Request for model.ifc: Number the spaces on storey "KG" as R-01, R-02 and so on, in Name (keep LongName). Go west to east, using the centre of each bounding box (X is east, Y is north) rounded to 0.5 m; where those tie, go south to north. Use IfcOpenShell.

First a look at what the model holds.

```python
import ifcopenshell
import ifcopenshell.util.element
import ifcopenshell.util.placement

model = ifcopenshell.open("model.ifc")
print(model.schema)
storey = next(s for s in model.by_type("IfcBuildingStorey") if s.Name == "KG")
spaces = [e for e in ifcopenshell.util.element.get_decomposition(storey) if e.is_a("IfcSpace")]
for e in sorted(spaces, key=lambda e: e.id()):
    origin = ifcopenshell.util.placement.get_local_placement(e.ObjectPlacement)[:3, 3]
    print(e.id(), e.Name, e.LongName, origin.round(2) + 0.0, sep=" | ")
```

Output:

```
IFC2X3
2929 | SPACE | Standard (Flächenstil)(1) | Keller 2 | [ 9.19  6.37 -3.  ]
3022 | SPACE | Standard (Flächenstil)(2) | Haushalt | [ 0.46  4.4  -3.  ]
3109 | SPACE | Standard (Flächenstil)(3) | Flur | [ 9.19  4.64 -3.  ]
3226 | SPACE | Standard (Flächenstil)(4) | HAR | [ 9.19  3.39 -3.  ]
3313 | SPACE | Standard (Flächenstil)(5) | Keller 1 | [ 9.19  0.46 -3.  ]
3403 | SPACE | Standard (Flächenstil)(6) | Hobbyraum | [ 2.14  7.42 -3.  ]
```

```python
import ifcopenshell
import ifcopenshell.geom
import ifcopenshell.util.element
import ifcopenshell.util.shape

model = ifcopenshell.open("model.ifc")
settings = ifcopenshell.geom.settings()
settings.set("use-world-coords", True)


def centre(element):
    shape = ifcopenshell.geom.create_shape(settings, element)
    return ifcopenshell.util.shape.get_bbox_centroid(shape.geometry)


storey = next(s for s in model.by_type("IfcBuildingStorey") if s.Name == "KG")
spaces = [e for e in ifcopenshell.util.element.get_decomposition(storey) if e.is_a("IfcSpace")]

# Insertion points can sit at a corner or the storey origin, so sort by the geometry (in metres).
centres = {e: centre(e) for e in spaces}
spaces.sort(key=lambda e: (round(centres[e][0] / 0.5), centres[e][1]))

for i, e in enumerate(spaces, start=1):
    number = f"R-{i:02d}"
    e.Name = number
    print(e.id(), number)

model.write("model_edited.ifc")
```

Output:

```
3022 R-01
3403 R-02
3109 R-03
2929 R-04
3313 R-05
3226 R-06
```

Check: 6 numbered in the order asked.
